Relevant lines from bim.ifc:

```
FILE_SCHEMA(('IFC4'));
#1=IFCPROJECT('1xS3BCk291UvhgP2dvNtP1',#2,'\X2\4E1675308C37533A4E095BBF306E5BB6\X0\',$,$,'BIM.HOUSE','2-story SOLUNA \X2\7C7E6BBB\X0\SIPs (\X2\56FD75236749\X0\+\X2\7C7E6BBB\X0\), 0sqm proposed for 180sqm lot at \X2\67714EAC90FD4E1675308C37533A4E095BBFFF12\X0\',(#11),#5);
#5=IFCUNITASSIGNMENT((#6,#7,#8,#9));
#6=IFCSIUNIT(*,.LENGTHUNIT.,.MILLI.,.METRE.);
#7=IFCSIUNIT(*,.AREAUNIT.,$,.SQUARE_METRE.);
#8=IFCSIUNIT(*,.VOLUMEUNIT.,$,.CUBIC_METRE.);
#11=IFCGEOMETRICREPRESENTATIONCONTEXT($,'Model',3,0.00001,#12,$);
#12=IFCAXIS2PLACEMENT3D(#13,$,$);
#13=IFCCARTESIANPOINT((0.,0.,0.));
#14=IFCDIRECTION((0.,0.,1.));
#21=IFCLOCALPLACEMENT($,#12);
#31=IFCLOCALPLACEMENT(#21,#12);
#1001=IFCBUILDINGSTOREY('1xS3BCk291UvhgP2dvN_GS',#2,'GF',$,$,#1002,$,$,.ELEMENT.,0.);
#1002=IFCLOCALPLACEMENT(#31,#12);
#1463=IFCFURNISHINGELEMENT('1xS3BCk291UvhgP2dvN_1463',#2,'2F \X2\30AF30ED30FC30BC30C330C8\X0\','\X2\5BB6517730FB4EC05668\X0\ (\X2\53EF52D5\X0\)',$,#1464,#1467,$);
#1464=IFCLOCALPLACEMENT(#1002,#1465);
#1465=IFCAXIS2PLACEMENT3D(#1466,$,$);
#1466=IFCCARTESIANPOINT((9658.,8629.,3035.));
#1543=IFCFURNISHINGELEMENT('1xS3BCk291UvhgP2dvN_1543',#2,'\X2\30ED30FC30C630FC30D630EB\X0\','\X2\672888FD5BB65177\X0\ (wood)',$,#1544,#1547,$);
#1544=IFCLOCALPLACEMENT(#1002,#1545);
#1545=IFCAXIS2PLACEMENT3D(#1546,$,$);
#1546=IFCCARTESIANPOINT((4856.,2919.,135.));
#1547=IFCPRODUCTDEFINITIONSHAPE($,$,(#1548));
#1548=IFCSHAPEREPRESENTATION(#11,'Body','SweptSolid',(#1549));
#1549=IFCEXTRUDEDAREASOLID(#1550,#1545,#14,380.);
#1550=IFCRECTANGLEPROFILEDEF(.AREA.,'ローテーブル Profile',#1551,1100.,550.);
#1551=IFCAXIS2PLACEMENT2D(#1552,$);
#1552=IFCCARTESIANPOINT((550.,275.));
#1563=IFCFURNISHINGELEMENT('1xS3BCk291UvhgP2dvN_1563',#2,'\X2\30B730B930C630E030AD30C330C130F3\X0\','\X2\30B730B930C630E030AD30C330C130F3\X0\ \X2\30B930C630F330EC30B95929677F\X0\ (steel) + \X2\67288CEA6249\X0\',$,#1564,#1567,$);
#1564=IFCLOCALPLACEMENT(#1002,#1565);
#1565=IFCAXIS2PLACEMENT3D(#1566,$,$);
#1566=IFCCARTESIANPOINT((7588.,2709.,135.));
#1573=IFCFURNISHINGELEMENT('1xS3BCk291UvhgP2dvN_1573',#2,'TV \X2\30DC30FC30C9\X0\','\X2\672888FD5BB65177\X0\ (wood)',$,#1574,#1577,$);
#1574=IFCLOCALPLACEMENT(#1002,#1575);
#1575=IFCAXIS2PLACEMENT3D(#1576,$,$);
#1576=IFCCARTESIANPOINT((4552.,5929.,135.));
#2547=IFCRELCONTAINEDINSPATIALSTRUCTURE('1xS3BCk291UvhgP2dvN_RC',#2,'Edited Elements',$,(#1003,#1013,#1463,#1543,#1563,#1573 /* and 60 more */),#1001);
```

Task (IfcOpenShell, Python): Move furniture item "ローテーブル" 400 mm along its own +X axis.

```python
import ifcopenshell
import ifcopenshell.api.geometry
import ifcopenshell.util.placement

model = ifcopenshell.open("bim.ifc")

item = model.by_guid("1xS3BCk291UvhgP2dvN_1543")
matrix = ifcopenshell.util.placement.get_local_placement(item.ObjectPlacement)
matrix[:3, 3] += matrix[:3, 0] * 400.0
ifcopenshell.api.geometry.edit_object_placement(model, product=item, matrix=matrix, is_si=False)

print(ifcopenshell.util.placement.get_local_placement(item.ObjectPlacement).round(3) + 0.0)

model.write("bim_v2.ifc")
```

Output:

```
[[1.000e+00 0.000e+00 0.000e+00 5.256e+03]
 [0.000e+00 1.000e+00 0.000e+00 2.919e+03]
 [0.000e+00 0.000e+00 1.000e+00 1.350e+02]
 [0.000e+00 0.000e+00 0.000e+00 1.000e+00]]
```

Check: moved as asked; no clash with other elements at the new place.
